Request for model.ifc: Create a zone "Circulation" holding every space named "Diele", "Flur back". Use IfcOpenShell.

First a look at what the model holds.

```python
import ifcopenshell

model = ifcopenshell.open("model.ifc")
print(model.schema)
seen = {}
for space in model.by_type("IfcSpace"):
    seen[space.LongName] = seen.get(space.LongName, 0) + 1
for name, count in sorted(seen.items(), key=str):
    print(count, "x", name)
print("zones:", [z.Name for z in model.by_type("IfcZone")][:20])
```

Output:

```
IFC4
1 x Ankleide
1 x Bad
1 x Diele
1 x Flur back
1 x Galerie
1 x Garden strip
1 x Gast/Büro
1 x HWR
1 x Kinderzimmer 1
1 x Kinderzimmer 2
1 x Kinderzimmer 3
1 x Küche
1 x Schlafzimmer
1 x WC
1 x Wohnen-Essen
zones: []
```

```python
import ifcopenshell
import ifcopenshell.api.group
import ifcopenshell.api.root

model = ifcopenshell.open("model.ifc")

names = {"Diele", "Flur back"}
spaces = [s for s in model.by_type("IfcSpace") if s.LongName in names]

zone = ifcopenshell.api.root.create_entity(model, ifc_class="IfcZone", name="Circulation")
ifcopenshell.api.group.assign_group(model, products=spaces, group=zone)
print(len(spaces), "spaces in", zone.Name)

model.write("model_edited.ifc")
```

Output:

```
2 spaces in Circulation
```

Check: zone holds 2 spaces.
